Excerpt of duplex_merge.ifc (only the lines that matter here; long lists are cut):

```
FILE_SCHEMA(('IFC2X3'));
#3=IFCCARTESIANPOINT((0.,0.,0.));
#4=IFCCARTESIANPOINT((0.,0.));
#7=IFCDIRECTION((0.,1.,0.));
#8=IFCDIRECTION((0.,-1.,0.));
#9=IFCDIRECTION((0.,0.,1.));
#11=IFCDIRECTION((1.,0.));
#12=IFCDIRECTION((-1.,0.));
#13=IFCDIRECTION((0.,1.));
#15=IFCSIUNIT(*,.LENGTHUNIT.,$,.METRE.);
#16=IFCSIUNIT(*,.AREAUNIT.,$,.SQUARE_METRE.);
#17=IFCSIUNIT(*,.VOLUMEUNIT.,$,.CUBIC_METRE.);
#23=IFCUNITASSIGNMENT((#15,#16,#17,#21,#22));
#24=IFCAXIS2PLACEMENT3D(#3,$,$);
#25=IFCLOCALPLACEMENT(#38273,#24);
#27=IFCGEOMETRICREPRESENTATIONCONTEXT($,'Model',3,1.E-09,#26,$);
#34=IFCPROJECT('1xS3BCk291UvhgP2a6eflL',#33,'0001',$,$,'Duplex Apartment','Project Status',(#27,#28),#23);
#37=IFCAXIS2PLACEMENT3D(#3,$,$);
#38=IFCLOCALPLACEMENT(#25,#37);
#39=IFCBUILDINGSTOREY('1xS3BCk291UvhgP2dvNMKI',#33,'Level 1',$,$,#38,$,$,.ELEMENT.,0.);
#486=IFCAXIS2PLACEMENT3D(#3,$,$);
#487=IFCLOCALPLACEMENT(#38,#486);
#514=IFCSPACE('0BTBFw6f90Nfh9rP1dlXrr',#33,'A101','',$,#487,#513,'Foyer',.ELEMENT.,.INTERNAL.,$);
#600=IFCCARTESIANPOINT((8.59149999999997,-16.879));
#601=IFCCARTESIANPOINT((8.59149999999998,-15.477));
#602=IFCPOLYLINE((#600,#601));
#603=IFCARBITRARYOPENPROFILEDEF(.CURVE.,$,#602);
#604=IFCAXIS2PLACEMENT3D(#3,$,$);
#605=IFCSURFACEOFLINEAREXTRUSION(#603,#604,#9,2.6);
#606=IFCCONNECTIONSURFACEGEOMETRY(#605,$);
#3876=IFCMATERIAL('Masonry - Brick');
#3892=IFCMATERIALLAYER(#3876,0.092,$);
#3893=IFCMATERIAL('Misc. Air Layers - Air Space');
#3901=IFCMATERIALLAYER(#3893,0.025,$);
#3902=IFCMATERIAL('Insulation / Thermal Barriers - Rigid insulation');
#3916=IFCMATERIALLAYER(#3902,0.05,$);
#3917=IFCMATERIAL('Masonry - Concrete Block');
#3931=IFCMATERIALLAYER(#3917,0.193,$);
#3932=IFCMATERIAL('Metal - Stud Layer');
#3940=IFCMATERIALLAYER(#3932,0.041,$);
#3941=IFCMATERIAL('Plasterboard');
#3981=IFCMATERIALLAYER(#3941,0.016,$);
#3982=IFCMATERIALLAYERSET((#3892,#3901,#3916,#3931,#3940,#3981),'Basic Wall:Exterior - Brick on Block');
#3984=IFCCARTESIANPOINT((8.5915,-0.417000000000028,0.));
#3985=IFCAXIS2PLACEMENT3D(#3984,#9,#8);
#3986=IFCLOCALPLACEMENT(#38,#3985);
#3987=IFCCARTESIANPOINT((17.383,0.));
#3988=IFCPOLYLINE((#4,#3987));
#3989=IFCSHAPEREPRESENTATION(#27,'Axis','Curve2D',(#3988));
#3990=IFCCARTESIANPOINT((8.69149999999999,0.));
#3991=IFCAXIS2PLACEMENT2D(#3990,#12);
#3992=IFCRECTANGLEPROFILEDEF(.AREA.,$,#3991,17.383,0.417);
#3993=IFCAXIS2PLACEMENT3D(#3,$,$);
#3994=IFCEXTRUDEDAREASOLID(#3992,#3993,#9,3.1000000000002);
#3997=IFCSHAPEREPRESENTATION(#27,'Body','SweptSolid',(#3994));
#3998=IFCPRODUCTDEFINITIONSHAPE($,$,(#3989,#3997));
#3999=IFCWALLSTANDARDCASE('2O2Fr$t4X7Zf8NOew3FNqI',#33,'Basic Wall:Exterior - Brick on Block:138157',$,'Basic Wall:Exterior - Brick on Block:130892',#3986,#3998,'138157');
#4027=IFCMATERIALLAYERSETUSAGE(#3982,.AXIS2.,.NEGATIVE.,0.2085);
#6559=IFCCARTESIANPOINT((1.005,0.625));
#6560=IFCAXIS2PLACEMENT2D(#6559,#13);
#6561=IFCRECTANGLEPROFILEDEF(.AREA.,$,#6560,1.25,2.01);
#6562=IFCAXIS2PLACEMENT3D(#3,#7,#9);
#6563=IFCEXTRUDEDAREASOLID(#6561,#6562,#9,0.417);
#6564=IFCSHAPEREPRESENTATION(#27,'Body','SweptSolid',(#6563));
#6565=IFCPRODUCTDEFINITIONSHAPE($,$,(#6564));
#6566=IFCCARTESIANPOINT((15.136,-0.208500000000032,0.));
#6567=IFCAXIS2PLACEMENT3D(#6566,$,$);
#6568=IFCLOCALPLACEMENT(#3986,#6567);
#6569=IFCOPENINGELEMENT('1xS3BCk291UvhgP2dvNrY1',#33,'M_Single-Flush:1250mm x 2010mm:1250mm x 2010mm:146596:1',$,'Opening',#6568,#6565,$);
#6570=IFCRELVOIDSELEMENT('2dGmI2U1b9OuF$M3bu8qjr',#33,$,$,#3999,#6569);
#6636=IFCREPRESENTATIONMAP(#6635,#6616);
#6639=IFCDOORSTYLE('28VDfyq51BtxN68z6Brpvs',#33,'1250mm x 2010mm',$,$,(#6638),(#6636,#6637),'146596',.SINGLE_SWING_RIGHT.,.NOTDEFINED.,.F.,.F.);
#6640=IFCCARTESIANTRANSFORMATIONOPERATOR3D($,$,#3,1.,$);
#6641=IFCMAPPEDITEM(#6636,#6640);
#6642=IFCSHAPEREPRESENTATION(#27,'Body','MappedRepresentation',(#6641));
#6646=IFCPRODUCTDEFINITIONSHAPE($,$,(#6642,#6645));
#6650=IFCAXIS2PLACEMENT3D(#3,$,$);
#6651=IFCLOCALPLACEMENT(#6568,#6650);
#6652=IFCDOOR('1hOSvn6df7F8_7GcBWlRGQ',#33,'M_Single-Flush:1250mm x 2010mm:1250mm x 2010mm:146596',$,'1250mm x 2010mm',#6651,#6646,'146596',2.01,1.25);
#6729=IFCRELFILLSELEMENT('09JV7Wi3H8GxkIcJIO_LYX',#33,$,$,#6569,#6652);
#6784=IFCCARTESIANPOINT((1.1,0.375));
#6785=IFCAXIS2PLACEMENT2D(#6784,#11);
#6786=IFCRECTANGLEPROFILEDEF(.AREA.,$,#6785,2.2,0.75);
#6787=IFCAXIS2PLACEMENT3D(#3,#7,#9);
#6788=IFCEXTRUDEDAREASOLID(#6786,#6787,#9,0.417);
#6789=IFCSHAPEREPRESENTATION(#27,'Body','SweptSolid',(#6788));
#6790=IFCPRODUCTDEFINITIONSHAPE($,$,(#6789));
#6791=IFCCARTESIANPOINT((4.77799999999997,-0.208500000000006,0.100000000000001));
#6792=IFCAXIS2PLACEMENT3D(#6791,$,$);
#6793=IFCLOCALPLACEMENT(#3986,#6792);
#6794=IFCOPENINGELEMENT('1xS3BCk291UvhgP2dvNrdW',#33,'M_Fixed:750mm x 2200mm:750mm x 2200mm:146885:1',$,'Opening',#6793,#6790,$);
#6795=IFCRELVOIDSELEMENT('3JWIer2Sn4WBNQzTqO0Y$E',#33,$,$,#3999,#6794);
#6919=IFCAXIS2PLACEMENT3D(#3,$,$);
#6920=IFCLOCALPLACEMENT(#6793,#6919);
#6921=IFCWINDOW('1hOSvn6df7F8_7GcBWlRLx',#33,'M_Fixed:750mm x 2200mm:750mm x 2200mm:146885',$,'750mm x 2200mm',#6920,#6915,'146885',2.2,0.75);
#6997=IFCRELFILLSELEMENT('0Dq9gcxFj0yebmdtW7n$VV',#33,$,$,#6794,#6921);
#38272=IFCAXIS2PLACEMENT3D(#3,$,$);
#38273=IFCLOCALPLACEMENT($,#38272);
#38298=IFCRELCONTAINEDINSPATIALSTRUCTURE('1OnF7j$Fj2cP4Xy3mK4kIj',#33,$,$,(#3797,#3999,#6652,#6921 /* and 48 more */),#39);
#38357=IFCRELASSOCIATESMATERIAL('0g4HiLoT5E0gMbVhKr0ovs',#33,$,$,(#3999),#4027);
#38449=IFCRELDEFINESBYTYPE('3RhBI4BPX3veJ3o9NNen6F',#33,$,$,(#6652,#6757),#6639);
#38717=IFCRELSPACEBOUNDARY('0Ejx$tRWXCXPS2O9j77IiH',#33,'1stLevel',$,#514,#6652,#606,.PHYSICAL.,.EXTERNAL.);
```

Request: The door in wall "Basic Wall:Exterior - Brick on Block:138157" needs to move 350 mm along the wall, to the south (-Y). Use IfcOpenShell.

```python
import numpy as np
import ifcopenshell
import ifcopenshell.api.geometry
import ifcopenshell.util.placement
import ifcopenshell.util.unit

model = ifcopenshell.open("duplex_merge.ifc")
unit_scale = ifcopenshell.util.unit.calculate_unit_scale(model)

door = model.by_guid("1hOSvn6df7F8_7GcBWlRGQ")
opening = door.FillsVoids[0].RelatingOpeningElement
wall = opening.VoidsElements[0].RelatingBuildingElement

wall_matrix = ifcopenshell.util.placement.get_local_placement(wall.ObjectPlacement)
shift = wall_matrix[:3, 0] * 0.35 / unit_scale
before = ifcopenshell.util.placement.get_local_placement(door.ObjectPlacement)[:3, 3].copy()

# The door is placed relative to its opening, so it follows when the opening moves.
matrix = ifcopenshell.util.placement.get_local_placement(opening.ObjectPlacement)
matrix[:3, 3] += shift
ifcopenshell.api.geometry.edit_object_placement(
    model, product=opening, matrix=matrix, is_si=False, should_transform_children=True
)

# Space boundary surfaces are stored in each space's coordinates; move them too.
for rel in door.ProvidesBoundaries:
    if not rel.ConnectionGeometry:
        continue
    surface = rel.ConnectionGeometry.SurfaceOnRelatingElement
    space_matrix = ifcopenshell.util.placement.get_local_placement(rel.RelatingSpace.ObjectPlacement)
    point = np.array(surface.Position.Location.Coordinates) + space_matrix[:3, :3].T @ shift
    surface.Position = model.createIfcAxis2Placement3D(
        model.createIfcCartesianPoint(point.tolist()), surface.Position.Axis, surface.Position.RefDirection
    )

after = ifcopenshell.util.placement.get_local_placement(door.ObjectPlacement)[:3, 3]
print("door moved by", (after - before).round(3) + 0.0)

model.write("duplex_merge_rev.ifc")
```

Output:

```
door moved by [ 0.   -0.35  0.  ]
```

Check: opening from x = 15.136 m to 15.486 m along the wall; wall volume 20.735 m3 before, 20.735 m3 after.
